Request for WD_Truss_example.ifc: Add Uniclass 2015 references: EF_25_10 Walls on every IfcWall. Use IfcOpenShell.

First a look at what the model holds.

```python
import ifcopenshell

model = ifcopenshell.open("WD_Truss_example.ifc")
print(model.schema)
print("classifications:", [c.Name for c in model.by_type("IfcClassification")])
for ifc_class in ("IfcDoor", "IfcRoof", "IfcStair", "IfcWall", "IfcWindow"):
    print(ifc_class, len(model.by_type(ifc_class)))
```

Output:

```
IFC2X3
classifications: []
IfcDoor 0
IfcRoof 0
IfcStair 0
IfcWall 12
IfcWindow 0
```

```python
import ifcopenshell
import ifcopenshell.api.classification

model = ifcopenshell.open("WD_Truss_example.ifc")

# IFC2X3 requires Source and Edition and has no link from the project to the system.
system = model.create_entity("IfcClassification", Source="NBS", Edition="2015", Name="Uniclass 2015")

codes = {
    "IfcWall": ("EF_25_10", "Walls"),
}
for ifc_class, (code, name) in codes.items():
    products = model.by_type(ifc_class)
    ifcopenshell.api.classification.add_reference(
        model, products=products, classification=system, identification=code, name=name
    )
    print(code, len(products))

model.write("WD_Truss_example_edited.ifc")
```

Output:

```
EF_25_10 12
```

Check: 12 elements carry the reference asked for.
